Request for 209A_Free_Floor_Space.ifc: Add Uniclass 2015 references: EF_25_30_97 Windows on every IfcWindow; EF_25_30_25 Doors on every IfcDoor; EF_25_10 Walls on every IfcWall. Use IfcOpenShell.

First a look at what the model holds.

```python
import ifcopenshell

model = ifcopenshell.open("209A_Free_Floor_Space.ifc")
print(model.schema)
print("classifications:", [c.Name for c in model.by_type("IfcClassification")])
for ifc_class in ("IfcDoor", "IfcRoof", "IfcStair", "IfcWall", "IfcWindow"):
    print(ifc_class, len(model.by_type(ifc_class)))
```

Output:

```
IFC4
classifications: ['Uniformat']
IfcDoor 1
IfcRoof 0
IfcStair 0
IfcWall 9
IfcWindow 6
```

```python
import ifcopenshell
import ifcopenshell.api.classification

model = ifcopenshell.open("209A_Free_Floor_Space.ifc")

system = ifcopenshell.api.classification.add_classification(model, classification="Uniclass 2015")

codes = {
    "IfcWindow": ("EF_25_30_97", "Windows"),
    "IfcDoor": ("EF_25_30_25", "Doors"),
    "IfcWall": ("EF_25_10", "Walls"),
}
for ifc_class, (code, name) in codes.items():
    products = model.by_type(ifc_class)
    ifcopenshell.api.classification.add_reference(
        model, products=products, classification=system, identification=code, name=name
    )
    print(code, len(products))

model.write("209A_Free_Floor_Space_rev.ifc")
```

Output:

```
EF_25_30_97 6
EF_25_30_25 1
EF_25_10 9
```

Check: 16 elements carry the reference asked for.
